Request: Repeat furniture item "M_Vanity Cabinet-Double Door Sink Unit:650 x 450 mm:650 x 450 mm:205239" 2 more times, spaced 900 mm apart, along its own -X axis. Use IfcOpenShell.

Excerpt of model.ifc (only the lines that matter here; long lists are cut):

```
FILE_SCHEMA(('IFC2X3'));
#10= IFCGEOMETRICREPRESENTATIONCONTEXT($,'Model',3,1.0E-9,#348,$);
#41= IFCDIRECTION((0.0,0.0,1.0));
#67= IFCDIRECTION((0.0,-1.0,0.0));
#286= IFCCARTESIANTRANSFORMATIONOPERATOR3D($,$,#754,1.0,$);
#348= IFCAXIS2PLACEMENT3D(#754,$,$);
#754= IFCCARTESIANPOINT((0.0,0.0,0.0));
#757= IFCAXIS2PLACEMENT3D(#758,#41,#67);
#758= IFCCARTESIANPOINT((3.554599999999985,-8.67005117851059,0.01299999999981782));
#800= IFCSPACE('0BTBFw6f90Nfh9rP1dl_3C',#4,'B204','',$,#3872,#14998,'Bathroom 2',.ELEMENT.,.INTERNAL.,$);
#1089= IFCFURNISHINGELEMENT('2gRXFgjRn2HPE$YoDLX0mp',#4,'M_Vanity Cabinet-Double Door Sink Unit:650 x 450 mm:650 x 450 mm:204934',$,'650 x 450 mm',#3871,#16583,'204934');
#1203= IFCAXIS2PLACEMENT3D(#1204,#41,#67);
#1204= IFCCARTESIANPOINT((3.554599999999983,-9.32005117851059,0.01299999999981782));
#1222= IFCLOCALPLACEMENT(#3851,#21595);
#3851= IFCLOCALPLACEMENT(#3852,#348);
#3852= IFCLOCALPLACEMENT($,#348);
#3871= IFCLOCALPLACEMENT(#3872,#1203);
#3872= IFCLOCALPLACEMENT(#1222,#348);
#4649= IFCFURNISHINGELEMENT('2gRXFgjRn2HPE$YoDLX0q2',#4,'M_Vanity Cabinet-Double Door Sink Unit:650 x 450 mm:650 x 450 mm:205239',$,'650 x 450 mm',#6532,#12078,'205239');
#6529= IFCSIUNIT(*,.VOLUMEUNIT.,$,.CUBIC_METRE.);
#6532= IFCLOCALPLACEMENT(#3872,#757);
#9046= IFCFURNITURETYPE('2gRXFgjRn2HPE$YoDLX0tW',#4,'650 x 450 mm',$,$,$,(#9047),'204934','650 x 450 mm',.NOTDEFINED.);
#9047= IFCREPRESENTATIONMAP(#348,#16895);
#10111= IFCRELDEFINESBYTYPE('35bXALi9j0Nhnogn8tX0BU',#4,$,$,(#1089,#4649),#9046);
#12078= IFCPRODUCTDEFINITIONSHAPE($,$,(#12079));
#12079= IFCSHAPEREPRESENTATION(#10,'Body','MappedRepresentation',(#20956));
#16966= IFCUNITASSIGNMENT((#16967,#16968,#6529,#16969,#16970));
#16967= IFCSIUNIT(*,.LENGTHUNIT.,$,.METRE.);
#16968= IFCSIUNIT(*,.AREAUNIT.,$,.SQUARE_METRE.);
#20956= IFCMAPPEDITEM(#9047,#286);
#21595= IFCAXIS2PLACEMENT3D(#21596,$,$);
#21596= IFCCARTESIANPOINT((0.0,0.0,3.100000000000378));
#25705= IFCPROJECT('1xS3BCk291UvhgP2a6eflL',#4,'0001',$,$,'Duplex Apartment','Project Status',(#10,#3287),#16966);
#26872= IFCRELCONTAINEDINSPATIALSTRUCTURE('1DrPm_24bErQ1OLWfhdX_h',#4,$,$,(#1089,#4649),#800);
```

```python
import ifcopenshell
import ifcopenshell.api.geometry
import ifcopenshell.api.root
import ifcopenshell.util.element
import ifcopenshell.util.placement
import ifcopenshell.util.unit

model = ifcopenshell.open("model.ifc")
unit_scale = ifcopenshell.util.unit.calculate_unit_scale(model)


def reuse_history(source, copy):
    """copy_class also copies each property set's owner history, people and application; keep the originals."""
    for rel in copy.IsDefinedBy:
        if rel.is_a("IfcRelDefinesByProperties") and (history := rel.RelatingPropertyDefinition.OwnerHistory):
            rel.RelatingPropertyDefinition.OwnerHistory = source.OwnerHistory
            ifcopenshell.util.element.remove_deep2(model, history)


source = model.by_guid("2gRXFgjRn2HPE$YoDLX0q2")
base = ifcopenshell.util.placement.get_local_placement(source.ObjectPlacement)
step = -base[:3, 0] * 0.9 / unit_scale

for i in range(1, 3):
    copy = ifcopenshell.api.root.copy_class(model, product=source)
    copy.Representation = ifcopenshell.util.element.copy_deep(
        model, source.Representation, exclude=["IfcGeometricRepresentationContext", "IfcRepresentationMap"]
    )
    copy.Name = "M_Vanity Cabinet-Double Door Sink Unit:650 x 450 mm:650 x 450 mm"
    copy.Tag = None
    reuse_history(source, copy)
    matrix = base.copy()
    matrix[:3, 3] += i * step
    print("added at", matrix[:3, 3].round(3) + 0.0)
    ifcopenshell.api.geometry.edit_object_placement(model, product=copy, matrix=matrix, is_si=False)

model.write("model_edited.ifc")
```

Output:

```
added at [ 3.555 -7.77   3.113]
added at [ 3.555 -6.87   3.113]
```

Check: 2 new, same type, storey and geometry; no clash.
